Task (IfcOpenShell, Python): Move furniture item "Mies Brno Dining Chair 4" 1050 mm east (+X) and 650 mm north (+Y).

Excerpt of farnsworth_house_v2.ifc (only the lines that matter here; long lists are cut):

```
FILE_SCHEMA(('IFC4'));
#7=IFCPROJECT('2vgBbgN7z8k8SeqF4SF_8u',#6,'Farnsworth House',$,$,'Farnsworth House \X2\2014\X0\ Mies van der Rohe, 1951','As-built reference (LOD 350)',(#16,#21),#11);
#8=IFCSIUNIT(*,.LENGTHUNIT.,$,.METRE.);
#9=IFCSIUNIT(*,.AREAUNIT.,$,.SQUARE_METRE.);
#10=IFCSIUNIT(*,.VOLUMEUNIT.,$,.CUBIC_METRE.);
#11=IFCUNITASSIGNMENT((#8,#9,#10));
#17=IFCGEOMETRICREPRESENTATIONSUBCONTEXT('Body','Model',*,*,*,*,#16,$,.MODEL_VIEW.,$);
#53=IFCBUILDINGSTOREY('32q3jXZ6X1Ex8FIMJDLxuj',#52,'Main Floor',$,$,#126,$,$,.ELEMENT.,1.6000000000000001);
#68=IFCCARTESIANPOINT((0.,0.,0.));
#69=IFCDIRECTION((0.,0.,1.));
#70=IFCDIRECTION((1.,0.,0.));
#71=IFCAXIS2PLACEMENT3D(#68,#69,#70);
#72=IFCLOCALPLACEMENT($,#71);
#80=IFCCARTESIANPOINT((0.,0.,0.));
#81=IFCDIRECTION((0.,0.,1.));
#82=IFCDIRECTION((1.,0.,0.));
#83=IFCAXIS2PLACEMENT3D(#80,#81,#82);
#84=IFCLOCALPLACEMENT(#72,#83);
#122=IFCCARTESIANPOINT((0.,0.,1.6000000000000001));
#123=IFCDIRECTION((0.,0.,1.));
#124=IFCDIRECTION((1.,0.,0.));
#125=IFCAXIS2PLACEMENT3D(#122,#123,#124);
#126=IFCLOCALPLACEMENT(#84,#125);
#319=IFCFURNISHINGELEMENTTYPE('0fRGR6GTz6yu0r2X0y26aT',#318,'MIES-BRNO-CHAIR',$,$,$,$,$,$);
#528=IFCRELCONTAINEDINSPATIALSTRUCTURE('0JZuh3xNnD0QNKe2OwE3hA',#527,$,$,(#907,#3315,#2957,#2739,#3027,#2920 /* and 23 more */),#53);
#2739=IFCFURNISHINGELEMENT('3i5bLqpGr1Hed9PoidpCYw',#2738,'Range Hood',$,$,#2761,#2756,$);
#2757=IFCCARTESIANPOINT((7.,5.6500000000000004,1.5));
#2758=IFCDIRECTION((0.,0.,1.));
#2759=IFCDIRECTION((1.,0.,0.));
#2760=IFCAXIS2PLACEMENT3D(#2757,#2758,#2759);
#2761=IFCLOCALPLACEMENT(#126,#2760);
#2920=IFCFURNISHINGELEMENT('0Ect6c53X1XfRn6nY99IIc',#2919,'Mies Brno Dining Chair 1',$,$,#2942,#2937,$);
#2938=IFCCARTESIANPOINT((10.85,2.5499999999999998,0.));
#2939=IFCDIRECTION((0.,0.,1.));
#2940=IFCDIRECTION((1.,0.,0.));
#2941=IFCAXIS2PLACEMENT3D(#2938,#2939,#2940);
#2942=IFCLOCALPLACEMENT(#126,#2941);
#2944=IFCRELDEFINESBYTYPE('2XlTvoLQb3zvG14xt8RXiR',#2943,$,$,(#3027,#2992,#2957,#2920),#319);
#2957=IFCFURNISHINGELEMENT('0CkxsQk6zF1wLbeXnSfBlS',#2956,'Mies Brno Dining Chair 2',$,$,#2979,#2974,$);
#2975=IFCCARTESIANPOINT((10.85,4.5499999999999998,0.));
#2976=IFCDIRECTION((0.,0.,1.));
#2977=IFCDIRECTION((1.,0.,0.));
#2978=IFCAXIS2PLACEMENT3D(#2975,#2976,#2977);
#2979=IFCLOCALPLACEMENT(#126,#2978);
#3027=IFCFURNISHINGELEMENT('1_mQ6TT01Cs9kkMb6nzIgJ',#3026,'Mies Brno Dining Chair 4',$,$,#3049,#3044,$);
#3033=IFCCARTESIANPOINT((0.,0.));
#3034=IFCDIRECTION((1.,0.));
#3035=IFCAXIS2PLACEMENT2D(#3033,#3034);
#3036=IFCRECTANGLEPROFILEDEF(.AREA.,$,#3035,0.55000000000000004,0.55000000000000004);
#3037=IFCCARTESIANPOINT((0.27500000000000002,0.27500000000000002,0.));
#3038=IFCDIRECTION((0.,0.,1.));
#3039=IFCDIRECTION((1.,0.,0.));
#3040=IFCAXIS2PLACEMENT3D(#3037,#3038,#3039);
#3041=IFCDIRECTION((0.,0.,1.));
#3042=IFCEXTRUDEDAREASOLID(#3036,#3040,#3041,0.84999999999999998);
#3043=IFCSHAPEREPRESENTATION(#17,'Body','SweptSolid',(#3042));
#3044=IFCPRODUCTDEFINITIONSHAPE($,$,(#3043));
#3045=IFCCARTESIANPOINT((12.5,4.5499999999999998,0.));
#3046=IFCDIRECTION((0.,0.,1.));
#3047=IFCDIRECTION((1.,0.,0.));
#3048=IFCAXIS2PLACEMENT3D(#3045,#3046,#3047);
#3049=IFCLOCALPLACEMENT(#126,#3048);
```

```python
import ifcopenshell
import ifcopenshell.api.geometry
import ifcopenshell.util.placement

model = ifcopenshell.open("farnsworth_house_v2.ifc")

item = model.by_guid("1_mQ6TT01Cs9kkMb6nzIgJ")
matrix = ifcopenshell.util.placement.get_local_placement(item.ObjectPlacement)
matrix[0, 3] += 1.05
matrix[1, 3] += 0.65
ifcopenshell.api.geometry.edit_object_placement(model, product=item, matrix=matrix, is_si=False)

print(ifcopenshell.util.placement.get_local_placement(item.ObjectPlacement).round(3) + 0.0)

model.write("farnsworth_house_v2-out.ifc")
```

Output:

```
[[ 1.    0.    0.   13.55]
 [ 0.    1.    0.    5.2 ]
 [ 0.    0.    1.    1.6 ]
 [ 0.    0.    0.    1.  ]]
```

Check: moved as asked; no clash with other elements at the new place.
